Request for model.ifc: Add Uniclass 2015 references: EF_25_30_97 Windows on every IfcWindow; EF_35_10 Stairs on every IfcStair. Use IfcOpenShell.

First a look at what the model holds.

```python
import ifcopenshell

model = ifcopenshell.open("model.ifc")
print(model.schema)
print("classifications:", [c.Name for c in model.by_type("IfcClassification")])
for ifc_class in ("IfcDoor", "IfcRoof", "IfcStair", "IfcWall", "IfcWindow"):
    print(ifc_class, len(model.by_type(ifc_class)))
```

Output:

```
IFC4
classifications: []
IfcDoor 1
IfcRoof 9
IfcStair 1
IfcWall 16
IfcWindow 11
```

```python
import ifcopenshell
import ifcopenshell.api.classification

model = ifcopenshell.open("model.ifc")

system = ifcopenshell.api.classification.add_classification(model, classification="Uniclass 2015")

codes = {
    "IfcWindow": ("EF_25_30_97", "Windows"),
    "IfcStair": ("EF_35_10", "Stairs"),
}
for ifc_class, (code, name) in codes.items():
    products = model.by_type(ifc_class)
    ifcopenshell.api.classification.add_reference(
        model, products=products, classification=system, identification=code, name=name
    )
    print(code, len(products))

model.write("model_rev.ifc")
```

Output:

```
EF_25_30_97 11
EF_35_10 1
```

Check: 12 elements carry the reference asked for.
